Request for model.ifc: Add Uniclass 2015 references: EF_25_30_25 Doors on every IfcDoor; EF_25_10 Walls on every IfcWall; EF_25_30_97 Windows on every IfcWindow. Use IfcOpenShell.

First a look at what the model holds.

```python
import ifcopenshell

model = ifcopenshell.open("model.ifc")
print(model.schema)
print("classifications:", [c.Name for c in model.by_type("IfcClassification")])
for ifc_class in ("IfcDoor", "IfcRoof", "IfcStair", "IfcWall", "IfcWindow"):
    print(ifc_class, len(model.by_type(ifc_class)))
```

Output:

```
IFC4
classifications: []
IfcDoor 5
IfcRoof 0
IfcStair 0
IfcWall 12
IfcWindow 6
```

```python
import ifcopenshell
import ifcopenshell.api.classification

model = ifcopenshell.open("model.ifc")

system = ifcopenshell.api.classification.add_classification(model, classification="Uniclass 2015")

codes = {
    "IfcDoor": ("EF_25_30_25", "Doors"),
    "IfcWall": ("EF_25_10", "Walls"),
    "IfcWindow": ("EF_25_30_97", "Windows"),
}
for ifc_class, (code, name) in codes.items():
    products = model.by_type(ifc_class)
    ifcopenshell.api.classification.add_reference(
        model, products=products, classification=system, identification=code, name=name
    )
    print(code, len(products))

model.write("model_rev.ifc")
```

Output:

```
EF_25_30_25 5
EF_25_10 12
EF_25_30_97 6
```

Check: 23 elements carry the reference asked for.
